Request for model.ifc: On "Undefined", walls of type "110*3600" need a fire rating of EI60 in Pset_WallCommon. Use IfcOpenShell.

First a look at what the model holds.

```python
import ifcopenshell
import ifcopenshell.util.element

model = ifcopenshell.open("model.ifc")
print(model.schema)
storey = next(s for s in model.by_type("IfcBuildingStorey") if s.Name == "Undefined")
walls = [e for e in ifcopenshell.util.element.get_decomposition(storey) if e.is_a("IfcWall")]
seen = {}
for e in walls:
    element_type = ifcopenshell.util.element.get_type(e)
    key = (element_type.Name if element_type != e and element_type else None, ifcopenshell.util.element.get_pset(e, "Pset_WallCommon", "FireRating"))
    seen[key] = seen.get(key, 0) + 1
for (name, value), count in sorted(seen.items(), key=str):
    print(count, "x", name, "|", value)
```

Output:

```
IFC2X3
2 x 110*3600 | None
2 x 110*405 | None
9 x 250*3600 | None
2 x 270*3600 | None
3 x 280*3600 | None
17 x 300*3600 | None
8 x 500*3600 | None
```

```python
import ifcopenshell
import ifcopenshell.api.pset
import ifcopenshell.util.element

model = ifcopenshell.open("model.ifc")

storey = next(s for s in model.by_type("IfcBuildingStorey") if s.Name == "Undefined")
walls = [e for e in ifcopenshell.util.element.get_decomposition(storey) if e.is_a("IfcWall")]

count = 0
for e in walls:
    element_type = ifcopenshell.util.element.get_type(e)
    if element_type in (None, e) or element_type.Name != "110*3600":
        continue
    found = ifcopenshell.util.element.get_pset(e, "Pset_WallCommon", should_inherit=False)
    if found:
        pset = model.by_id(found["id"])
        if len(ifcopenshell.util.element.get_elements_by_pset(pset)) > 1:
            pset = ifcopenshell.api.pset.unshare_pset(model, products=[e], pset=pset)[0]
    else:
        pset = ifcopenshell.api.pset.add_pset(model, product=e, name="Pset_WallCommon")
    ifcopenshell.api.pset.edit_pset(model, pset=pset, properties={"FireRating": "EI60"})
    count += 1

print(count, "walls updated")

model.write("model_v2.ifc")
```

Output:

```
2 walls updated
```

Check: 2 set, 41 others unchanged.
